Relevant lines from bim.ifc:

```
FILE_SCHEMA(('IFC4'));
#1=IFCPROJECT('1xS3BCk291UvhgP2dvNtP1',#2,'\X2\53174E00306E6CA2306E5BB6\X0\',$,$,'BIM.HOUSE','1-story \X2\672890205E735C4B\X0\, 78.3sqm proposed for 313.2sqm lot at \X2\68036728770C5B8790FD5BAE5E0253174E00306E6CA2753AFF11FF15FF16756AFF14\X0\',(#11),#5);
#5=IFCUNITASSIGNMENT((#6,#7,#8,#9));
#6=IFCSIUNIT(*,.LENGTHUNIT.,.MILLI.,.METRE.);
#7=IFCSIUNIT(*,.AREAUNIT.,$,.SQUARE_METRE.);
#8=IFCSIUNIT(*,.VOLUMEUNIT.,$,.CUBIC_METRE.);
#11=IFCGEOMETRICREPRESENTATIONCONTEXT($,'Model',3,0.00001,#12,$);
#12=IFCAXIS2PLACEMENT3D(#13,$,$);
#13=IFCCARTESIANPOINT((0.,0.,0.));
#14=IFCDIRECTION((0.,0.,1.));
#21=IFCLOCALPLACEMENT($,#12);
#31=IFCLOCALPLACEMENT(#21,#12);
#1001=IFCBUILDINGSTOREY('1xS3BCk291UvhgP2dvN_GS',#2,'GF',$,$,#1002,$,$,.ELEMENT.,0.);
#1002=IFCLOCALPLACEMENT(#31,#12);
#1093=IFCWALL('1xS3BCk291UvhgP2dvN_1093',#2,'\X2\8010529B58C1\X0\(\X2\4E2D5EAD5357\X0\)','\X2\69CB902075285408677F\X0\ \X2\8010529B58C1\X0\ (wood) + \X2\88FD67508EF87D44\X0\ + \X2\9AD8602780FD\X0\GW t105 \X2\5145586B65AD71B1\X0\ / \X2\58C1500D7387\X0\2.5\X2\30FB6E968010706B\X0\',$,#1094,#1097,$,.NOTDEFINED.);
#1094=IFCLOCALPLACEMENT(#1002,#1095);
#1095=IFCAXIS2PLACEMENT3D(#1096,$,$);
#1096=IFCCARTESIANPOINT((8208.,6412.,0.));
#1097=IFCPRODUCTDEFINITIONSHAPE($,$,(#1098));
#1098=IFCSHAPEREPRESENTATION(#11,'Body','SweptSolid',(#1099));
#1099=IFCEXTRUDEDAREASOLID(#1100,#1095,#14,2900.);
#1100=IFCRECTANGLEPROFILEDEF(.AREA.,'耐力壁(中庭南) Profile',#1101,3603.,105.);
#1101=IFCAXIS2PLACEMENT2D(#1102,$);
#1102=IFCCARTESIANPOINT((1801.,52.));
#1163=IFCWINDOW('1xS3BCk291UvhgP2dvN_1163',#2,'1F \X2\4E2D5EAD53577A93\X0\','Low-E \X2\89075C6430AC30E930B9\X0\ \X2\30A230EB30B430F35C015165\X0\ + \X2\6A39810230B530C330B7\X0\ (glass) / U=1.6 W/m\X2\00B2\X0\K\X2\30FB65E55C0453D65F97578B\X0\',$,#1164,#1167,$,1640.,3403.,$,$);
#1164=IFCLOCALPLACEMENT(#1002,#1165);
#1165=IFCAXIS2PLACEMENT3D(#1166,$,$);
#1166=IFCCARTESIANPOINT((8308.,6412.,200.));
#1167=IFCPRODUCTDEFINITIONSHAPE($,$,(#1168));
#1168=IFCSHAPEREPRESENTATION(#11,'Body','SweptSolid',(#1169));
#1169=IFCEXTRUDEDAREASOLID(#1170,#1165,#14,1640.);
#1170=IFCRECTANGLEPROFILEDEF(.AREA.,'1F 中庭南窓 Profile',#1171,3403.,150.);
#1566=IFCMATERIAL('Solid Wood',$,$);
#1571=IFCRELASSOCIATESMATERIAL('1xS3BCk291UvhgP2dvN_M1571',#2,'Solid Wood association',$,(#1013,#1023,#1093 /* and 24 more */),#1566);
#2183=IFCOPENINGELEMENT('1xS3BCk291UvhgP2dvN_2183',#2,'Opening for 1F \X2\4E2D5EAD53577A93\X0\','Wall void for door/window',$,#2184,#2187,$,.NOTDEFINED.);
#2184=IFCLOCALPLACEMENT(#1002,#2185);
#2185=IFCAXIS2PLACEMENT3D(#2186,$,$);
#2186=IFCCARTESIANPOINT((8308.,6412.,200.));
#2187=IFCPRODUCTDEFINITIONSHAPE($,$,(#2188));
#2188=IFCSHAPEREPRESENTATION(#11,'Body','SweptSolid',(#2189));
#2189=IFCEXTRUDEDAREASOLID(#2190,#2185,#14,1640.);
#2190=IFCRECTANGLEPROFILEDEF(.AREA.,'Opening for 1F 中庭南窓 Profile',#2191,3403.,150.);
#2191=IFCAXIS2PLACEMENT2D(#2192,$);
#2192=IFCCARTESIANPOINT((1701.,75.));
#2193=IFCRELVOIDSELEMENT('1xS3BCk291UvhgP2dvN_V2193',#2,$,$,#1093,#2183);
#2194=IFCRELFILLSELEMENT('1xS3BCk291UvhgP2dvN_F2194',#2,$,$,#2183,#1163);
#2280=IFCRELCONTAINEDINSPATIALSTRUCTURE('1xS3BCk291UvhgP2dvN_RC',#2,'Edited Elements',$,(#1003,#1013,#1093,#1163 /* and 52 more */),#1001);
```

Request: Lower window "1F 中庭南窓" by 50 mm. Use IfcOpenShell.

```python
import numpy as np
import ifcopenshell
import ifcopenshell.api.geometry
import ifcopenshell.util.placement
import ifcopenshell.util.unit

model = ifcopenshell.open("bim.ifc")
unit_scale = ifcopenshell.util.unit.calculate_unit_scale(model)

window = model.by_guid("1xS3BCk291UvhgP2dvN_1163")
opening = window.FillsVoids[0].RelatingOpeningElement
dz = -0.05 / unit_scale

shift = np.array([0.0, 0.0, dz])
# The window is not placed relative to its opening, so move both.
for product in (opening, window):
    matrix = ifcopenshell.util.placement.get_local_placement(product.ObjectPlacement)
    matrix[:3, 3] += shift
    ifcopenshell.api.geometry.edit_object_placement(model, product=product, matrix=matrix, is_si=False)

print(f"moved by {dz * unit_scale:+.3f} m")

model.write("bim-out.ifc")
```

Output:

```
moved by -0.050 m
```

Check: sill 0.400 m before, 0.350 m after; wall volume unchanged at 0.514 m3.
